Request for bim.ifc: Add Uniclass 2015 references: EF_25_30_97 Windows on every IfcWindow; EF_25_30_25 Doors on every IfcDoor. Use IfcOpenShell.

First a look at what the model holds.

```python
import ifcopenshell

model = ifcopenshell.open("bim.ifc")
print(model.schema)
print("classifications:", [c.Name for c in model.by_type("IfcClassification")])
for ifc_class in ("IfcDoor", "IfcRoof", "IfcStair", "IfcWall", "IfcWindow"):
    print(ifc_class, len(model.by_type(ifc_class)))
```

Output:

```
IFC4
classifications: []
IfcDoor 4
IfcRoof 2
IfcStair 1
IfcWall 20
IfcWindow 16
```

```python
import ifcopenshell
import ifcopenshell.api.classification

model = ifcopenshell.open("bim.ifc")

system = ifcopenshell.api.classification.add_classification(model, classification="Uniclass 2015")

codes = {
    "IfcWindow": ("EF_25_30_97", "Windows"),
    "IfcDoor": ("EF_25_30_25", "Doors"),
}
for ifc_class, (code, name) in codes.items():
    products = model.by_type(ifc_class)
    ifcopenshell.api.classification.add_reference(
        model, products=products, classification=system, identification=code, name=name
    )
    print(code, len(products))

model.write("bim_rev.ifc")
```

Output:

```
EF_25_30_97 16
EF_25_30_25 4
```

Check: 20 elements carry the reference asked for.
